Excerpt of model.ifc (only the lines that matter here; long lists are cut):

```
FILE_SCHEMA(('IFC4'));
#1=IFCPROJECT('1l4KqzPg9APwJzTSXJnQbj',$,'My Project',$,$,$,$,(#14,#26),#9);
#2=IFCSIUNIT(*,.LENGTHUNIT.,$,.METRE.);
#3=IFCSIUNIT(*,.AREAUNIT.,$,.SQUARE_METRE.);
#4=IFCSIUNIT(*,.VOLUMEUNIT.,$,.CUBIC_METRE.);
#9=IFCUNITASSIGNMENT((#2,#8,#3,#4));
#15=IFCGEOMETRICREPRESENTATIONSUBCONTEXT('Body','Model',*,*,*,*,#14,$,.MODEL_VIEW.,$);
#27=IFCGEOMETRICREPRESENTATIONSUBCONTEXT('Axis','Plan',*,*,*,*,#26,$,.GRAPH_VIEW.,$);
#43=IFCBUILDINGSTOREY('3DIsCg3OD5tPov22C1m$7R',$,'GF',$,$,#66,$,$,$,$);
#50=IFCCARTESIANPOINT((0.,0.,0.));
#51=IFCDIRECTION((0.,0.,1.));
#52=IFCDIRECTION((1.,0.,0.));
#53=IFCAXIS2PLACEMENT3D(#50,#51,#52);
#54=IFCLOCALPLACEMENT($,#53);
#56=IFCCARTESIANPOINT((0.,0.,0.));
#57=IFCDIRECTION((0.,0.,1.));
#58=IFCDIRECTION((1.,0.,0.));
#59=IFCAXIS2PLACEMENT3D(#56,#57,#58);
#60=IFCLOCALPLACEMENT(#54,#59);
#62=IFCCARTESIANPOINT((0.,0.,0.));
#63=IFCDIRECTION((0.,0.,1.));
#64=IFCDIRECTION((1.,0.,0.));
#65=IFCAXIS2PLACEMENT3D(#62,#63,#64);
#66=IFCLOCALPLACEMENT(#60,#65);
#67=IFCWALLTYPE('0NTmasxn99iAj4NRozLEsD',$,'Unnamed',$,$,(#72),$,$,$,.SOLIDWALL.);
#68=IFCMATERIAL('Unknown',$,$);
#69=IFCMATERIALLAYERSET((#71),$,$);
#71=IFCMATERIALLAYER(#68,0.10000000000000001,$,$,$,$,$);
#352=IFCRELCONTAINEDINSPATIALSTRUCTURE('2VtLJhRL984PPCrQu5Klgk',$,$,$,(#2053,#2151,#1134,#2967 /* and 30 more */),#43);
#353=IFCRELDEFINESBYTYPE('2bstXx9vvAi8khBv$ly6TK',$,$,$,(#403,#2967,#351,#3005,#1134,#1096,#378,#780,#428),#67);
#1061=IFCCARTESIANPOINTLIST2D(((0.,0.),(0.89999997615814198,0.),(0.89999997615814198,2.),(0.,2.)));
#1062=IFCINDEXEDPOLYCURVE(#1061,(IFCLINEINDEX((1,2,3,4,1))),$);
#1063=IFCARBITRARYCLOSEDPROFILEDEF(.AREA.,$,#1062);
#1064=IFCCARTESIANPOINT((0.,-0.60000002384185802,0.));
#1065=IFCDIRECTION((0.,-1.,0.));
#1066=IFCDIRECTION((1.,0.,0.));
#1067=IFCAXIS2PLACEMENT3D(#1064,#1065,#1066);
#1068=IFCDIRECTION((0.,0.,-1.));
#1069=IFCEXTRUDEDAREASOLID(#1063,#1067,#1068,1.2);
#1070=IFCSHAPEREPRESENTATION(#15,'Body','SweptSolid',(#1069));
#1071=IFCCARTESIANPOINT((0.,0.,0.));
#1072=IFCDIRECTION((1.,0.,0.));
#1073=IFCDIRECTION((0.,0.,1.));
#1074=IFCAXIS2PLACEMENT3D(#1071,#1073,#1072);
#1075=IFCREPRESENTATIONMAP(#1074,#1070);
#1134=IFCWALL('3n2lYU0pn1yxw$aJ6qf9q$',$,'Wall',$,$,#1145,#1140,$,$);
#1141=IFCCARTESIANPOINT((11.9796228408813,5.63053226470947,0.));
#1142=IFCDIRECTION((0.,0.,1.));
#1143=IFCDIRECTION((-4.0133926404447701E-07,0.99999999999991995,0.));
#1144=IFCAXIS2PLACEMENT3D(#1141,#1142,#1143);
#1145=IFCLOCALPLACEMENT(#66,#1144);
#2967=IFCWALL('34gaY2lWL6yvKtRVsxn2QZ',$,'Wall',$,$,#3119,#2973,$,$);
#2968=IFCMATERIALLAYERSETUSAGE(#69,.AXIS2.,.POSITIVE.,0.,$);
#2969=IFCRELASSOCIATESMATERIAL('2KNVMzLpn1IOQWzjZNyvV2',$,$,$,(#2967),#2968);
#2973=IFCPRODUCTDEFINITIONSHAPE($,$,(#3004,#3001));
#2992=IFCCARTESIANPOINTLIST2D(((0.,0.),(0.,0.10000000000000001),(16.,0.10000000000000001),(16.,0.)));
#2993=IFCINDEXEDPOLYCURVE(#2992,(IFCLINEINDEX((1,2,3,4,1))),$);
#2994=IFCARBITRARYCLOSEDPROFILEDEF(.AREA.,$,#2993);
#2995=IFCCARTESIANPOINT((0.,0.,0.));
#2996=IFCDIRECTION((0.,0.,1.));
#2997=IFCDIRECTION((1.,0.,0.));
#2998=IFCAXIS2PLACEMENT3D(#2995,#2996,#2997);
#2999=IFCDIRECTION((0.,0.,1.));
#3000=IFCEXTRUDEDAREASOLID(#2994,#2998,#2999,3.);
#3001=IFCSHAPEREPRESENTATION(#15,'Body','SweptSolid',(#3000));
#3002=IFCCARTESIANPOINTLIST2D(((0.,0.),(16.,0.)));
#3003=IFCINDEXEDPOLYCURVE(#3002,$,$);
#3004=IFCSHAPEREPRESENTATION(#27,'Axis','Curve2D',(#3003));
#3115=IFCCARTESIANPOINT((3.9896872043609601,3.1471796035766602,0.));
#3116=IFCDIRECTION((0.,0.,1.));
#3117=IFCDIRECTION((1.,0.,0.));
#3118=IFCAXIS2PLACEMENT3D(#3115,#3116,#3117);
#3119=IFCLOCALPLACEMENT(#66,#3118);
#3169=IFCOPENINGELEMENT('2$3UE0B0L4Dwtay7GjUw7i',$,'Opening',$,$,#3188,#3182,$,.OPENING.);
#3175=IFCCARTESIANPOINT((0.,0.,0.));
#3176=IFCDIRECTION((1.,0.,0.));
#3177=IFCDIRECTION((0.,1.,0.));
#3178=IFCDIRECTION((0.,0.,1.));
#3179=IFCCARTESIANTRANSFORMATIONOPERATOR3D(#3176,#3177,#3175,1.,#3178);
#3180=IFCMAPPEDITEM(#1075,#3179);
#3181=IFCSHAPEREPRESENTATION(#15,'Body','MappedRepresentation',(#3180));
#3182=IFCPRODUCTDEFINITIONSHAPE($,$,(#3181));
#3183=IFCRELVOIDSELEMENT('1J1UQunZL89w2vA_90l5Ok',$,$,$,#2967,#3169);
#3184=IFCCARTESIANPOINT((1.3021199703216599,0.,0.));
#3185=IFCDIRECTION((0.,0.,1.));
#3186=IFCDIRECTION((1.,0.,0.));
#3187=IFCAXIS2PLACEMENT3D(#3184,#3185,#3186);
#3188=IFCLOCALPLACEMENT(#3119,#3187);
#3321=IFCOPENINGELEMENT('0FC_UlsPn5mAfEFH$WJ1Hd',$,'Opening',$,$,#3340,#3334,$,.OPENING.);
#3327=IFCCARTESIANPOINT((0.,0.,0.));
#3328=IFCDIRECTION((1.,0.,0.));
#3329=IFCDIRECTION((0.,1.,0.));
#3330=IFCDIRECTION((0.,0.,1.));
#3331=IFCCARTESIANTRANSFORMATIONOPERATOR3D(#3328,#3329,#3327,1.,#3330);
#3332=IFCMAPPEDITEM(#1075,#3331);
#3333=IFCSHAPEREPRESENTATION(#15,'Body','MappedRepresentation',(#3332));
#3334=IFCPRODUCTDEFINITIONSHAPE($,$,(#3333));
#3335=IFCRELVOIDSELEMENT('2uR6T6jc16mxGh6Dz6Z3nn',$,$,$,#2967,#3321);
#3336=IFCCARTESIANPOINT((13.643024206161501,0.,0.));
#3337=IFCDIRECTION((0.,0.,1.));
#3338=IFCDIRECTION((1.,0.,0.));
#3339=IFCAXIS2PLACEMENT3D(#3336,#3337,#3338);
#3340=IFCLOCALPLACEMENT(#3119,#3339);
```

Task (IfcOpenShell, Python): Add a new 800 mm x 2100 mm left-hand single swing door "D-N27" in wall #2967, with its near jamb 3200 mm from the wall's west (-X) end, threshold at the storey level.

```python
import numpy as np
import ifcopenshell
import ifcopenshell.api.feature
import ifcopenshell.api.geometry
import ifcopenshell.api.root
import ifcopenshell.api.spatial
import ifcopenshell.geom
import ifcopenshell.util.element
import ifcopenshell.util.placement
import ifcopenshell.util.representation
import ifcopenshell.util.shape
import ifcopenshell.util.unit

model = ifcopenshell.open("model.ifc")
unit_scale = ifcopenshell.util.unit.calculate_unit_scale(model)
settings = ifcopenshell.geom.settings()


def volume(element):
    """Net volume in cubic metres, openings subtracted."""
    shape = ifcopenshell.geom.create_shape(settings, element)
    return ifcopenshell.util.shape.get_volume(shape.geometry)


wall = model.by_guid("34gaY2lWL6yvKtRVsxn2QZ")
storey = ifcopenshell.util.element.get_container(wall, ifc_class="IfcBuildingStorey")
context = ifcopenshell.util.representation.get_context(model, "Model", "Body", "MODEL_VIEW")
before = volume(wall)

width, height, from_end, sill = 0.8, 2.1, 3.2, 0.0  # metres

# The wall runs along its own X axis, and the end named is its -X end.
wall_shape = ifcopenshell.geom.create_shape(settings, wall)
x, y, z = ifcopenshell.util.shape.get_vertices(wall_shape.geometry).T
start = x.min() + from_end
face, thickness = float(y.min()), float(y.max() - y.min())
wall_matrix = ifcopenshell.util.placement.get_local_placement(wall.ObjectPlacement)
level = ifcopenshell.util.placement.get_local_placement(storey.ObjectPlacement)[2, 3]


def in_wall(x, y):
    """Placement at x, y metres in the wall's axes, at sill height."""
    matrix = wall_matrix.copy()
    matrix[:, 3] = wall_matrix @ np.array([x / unit_scale, y / unit_scale, 0.0, 1.0])
    matrix[2, 3] = level + sill / unit_scale
    return matrix


# Opening: a box that overshoots both wall faces by 50 mm.
opening = ifcopenshell.api.root.create_entity(model, ifc_class="IfcOpeningElement", predefined_type="OPENING")
box = ifcopenshell.api.geometry.add_wall_representation(
    model, context=context, length=width, height=height, thickness=thickness + 0.1
)
ifcopenshell.api.geometry.assign_representation(model, product=opening, representation=box)
ifcopenshell.api.geometry.edit_object_placement(model, product=opening, matrix=in_wall(start, face - 0.05), is_si=False)
ifcopenshell.api.feature.add_feature(model, feature=opening, element=wall)

door = ifcopenshell.api.root.create_entity(model, ifc_class="IfcDoor", name="D-N27", predefined_type="DOOR")
door.OverallWidth, door.OverallHeight = width / unit_scale, height / unit_scale
door.OperationType = "SINGLE_SWING_LEFT"
body = ifcopenshell.api.geometry.add_door_representation(
    model,
    context=context,
    overall_width=door.OverallWidth,
    overall_height=door.OverallHeight,
    operation_type="SINGLE_SWING_LEFT",
    lining_properties={"LiningDepth": thickness / unit_scale, "ThresholdDepth": thickness / unit_scale},
)
ifcopenshell.api.geometry.assign_representation(model, product=door, representation=body)
ifcopenshell.api.spatial.assign_container(model, products=[door], relating_structure=storey)
ifcopenshell.api.feature.add_filling(model, opening=opening, element=door)

# The lining spans the wall, so the door starts at the wall face.
ifcopenshell.api.geometry.edit_object_placement(model, product=door, matrix=in_wall(start, face), is_si=False)

after = volume(wall)

print(f"wall volume {before:.3f} -> {after:.3f} m3")

model.write("model_rev.ifc")
```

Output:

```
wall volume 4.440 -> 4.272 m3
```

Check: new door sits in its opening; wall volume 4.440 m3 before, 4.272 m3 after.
